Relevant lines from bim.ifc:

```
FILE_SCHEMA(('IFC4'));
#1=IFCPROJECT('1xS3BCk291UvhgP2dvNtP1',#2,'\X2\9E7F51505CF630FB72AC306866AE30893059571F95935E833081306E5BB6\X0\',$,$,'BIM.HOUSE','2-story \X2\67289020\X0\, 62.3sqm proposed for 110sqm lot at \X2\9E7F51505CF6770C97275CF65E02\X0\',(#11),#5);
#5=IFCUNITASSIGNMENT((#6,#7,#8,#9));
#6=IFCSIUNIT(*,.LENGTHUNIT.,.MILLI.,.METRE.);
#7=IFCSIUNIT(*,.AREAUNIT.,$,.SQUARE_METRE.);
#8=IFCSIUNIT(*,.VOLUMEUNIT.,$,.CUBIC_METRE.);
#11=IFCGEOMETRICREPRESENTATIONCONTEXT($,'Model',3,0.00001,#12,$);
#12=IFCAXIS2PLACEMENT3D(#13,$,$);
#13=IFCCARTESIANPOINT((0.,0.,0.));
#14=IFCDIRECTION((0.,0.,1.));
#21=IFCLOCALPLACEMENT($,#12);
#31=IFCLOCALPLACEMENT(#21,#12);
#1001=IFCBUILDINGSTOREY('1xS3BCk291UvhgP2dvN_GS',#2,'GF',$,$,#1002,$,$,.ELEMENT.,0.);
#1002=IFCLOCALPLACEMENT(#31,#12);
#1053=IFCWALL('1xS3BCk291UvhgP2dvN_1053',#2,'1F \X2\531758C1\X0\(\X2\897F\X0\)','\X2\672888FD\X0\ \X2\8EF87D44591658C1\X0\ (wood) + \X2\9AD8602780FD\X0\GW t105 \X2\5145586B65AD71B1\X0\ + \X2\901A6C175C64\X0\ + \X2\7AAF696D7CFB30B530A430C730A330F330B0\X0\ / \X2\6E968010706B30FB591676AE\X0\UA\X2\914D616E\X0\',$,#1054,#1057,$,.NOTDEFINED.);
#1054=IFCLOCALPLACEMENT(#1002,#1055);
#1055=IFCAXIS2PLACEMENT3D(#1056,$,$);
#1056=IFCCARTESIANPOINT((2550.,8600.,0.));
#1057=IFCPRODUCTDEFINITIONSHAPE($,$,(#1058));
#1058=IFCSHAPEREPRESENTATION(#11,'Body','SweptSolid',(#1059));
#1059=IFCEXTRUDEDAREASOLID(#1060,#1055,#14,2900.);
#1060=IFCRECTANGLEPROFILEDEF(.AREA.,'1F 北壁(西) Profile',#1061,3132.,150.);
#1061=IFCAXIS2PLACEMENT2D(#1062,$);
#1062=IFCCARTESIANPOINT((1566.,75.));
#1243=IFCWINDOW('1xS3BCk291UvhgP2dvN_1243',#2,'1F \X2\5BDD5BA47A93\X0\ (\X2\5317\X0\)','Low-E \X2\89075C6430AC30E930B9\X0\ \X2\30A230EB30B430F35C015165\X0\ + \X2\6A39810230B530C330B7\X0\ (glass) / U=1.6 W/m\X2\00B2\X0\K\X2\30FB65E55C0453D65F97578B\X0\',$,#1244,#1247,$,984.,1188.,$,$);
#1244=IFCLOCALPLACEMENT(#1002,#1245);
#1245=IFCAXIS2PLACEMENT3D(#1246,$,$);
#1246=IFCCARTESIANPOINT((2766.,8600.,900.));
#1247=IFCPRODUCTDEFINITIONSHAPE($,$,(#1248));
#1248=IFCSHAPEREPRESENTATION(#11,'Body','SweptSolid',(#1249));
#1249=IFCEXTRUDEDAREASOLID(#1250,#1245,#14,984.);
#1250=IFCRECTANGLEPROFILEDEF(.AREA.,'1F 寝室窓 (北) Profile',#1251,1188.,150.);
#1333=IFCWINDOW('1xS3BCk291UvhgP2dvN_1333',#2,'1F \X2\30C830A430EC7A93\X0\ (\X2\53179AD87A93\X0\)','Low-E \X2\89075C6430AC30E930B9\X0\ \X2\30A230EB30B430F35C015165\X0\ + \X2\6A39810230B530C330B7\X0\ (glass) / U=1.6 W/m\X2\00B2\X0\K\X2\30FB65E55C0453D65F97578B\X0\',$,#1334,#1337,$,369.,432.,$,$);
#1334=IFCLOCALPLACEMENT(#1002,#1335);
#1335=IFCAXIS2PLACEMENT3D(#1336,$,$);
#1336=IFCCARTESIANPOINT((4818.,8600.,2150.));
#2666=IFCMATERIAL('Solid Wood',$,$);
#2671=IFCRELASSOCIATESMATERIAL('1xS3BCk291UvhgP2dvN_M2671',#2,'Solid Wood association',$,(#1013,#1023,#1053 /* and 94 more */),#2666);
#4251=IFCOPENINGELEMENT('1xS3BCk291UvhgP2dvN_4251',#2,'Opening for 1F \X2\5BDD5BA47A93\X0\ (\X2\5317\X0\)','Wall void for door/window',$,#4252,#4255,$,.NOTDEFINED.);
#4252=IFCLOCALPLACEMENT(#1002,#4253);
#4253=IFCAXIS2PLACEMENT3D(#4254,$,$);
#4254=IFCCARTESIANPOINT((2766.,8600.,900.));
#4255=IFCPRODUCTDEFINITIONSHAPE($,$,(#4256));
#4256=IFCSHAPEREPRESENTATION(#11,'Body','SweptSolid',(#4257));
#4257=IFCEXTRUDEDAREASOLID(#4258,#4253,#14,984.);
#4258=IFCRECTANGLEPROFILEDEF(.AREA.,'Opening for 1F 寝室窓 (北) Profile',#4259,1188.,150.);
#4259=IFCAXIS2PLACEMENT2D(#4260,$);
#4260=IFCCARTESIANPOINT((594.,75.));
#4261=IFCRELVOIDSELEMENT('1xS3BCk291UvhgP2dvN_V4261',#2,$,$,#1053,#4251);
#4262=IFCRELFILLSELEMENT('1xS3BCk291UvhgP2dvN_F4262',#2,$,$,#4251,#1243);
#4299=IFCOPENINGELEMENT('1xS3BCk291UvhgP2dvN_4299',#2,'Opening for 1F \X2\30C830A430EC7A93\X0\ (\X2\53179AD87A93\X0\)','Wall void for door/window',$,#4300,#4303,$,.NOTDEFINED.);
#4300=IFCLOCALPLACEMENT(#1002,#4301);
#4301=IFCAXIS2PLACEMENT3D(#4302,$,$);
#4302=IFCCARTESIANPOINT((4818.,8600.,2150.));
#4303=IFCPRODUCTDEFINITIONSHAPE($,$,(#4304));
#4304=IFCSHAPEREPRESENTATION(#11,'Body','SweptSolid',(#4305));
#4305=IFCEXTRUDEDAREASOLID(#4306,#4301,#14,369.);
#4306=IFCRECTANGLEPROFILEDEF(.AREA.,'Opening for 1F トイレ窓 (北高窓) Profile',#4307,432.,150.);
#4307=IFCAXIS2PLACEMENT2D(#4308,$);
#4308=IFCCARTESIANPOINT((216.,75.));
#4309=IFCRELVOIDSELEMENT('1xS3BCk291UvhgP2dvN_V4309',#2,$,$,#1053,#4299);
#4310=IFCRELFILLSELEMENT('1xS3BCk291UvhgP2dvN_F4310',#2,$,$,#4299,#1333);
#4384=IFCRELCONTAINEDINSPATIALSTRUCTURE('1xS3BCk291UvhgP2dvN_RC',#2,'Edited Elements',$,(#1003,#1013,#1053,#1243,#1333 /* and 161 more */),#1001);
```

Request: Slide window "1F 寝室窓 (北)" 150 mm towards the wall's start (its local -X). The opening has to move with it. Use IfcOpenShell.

```python
import ifcopenshell
import ifcopenshell.api.geometry
import ifcopenshell.util.placement
import ifcopenshell.util.unit

model = ifcopenshell.open("bim.ifc")
unit_scale = ifcopenshell.util.unit.calculate_unit_scale(model)

window = model.by_guid("1xS3BCk291UvhgP2dvN_1243")
opening = window.FillsVoids[0].RelatingOpeningElement
wall = opening.VoidsElements[0].RelatingBuildingElement

wall_matrix = ifcopenshell.util.placement.get_local_placement(wall.ObjectPlacement)
shift = wall_matrix[:3, 0] * -0.15 / unit_scale
before = ifcopenshell.util.placement.get_local_placement(window.ObjectPlacement)[:3, 3].copy()

# The window is not placed relative to its opening, so move both.
for product in (opening, window):
    matrix = ifcopenshell.util.placement.get_local_placement(product.ObjectPlacement)
    matrix[:3, 3] += shift
    ifcopenshell.api.geometry.edit_object_placement(model, product=product, matrix=matrix, is_si=False)

after = ifcopenshell.util.placement.get_local_placement(window.ObjectPlacement)[:3, 3]
print("window moved by", (after - before).round(3) + 0.0)

model.write("bim-out.ifc")
```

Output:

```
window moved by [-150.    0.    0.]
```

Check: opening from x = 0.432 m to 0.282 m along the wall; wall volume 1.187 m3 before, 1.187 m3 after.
